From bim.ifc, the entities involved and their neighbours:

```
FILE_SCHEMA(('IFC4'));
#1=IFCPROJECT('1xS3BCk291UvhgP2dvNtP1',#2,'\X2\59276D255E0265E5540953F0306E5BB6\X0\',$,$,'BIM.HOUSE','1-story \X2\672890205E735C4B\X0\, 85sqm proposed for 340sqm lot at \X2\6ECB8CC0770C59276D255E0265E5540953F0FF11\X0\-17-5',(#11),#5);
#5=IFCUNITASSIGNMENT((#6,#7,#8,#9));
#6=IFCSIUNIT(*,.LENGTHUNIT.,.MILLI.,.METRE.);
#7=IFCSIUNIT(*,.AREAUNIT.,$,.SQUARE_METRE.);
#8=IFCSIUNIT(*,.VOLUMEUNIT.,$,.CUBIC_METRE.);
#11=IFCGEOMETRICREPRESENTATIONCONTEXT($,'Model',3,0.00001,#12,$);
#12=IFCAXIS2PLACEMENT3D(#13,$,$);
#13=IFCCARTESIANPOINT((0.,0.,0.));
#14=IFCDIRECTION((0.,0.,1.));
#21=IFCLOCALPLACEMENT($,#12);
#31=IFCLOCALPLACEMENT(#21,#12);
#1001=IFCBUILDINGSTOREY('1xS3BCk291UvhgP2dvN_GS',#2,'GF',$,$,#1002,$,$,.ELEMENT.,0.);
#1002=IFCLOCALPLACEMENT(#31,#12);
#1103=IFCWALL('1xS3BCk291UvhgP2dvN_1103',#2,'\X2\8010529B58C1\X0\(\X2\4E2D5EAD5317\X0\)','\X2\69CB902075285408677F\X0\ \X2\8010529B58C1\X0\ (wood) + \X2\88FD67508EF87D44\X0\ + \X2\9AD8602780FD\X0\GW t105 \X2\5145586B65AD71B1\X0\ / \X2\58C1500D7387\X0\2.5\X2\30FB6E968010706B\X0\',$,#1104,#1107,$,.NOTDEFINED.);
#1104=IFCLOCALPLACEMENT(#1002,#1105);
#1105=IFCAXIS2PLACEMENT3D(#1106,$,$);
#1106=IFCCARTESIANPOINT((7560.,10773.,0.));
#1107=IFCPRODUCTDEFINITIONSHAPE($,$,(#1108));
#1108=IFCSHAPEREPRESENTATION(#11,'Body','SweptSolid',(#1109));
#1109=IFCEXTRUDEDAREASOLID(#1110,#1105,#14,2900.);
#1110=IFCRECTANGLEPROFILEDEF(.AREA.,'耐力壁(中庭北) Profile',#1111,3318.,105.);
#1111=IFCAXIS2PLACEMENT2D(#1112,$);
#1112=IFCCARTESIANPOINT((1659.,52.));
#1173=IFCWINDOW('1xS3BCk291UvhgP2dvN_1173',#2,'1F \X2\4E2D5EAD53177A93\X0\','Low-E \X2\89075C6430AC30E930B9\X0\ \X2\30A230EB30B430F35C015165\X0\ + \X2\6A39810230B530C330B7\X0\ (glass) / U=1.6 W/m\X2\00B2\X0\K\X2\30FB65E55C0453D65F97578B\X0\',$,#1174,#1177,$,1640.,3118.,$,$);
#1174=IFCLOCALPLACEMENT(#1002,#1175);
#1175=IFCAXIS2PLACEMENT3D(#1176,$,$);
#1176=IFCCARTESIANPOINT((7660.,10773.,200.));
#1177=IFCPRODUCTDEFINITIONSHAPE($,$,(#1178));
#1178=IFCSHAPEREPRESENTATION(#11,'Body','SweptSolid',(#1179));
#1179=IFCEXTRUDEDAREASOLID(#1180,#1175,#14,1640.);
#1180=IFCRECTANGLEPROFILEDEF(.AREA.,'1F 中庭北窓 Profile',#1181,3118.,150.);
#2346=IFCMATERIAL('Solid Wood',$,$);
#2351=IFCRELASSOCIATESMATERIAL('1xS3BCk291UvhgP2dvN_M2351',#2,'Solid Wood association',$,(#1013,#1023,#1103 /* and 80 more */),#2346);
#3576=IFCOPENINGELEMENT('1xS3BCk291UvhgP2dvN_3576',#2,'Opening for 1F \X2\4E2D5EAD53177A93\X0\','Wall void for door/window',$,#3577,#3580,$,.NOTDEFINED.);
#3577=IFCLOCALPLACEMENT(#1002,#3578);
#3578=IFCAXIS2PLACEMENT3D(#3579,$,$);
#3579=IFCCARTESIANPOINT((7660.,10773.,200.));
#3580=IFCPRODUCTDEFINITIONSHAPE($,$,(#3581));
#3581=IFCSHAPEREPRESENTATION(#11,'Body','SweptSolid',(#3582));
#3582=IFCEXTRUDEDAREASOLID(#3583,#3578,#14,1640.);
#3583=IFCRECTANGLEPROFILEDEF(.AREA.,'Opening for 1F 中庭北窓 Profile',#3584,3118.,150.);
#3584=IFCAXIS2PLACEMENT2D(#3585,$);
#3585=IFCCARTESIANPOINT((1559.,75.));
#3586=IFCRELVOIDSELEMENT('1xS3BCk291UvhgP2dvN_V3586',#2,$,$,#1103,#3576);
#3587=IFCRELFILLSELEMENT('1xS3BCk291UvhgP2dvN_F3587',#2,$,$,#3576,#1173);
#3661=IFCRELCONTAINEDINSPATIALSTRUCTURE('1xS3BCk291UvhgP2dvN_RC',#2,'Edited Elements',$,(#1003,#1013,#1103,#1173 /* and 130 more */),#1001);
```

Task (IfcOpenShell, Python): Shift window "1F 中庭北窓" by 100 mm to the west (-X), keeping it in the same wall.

```python
import ifcopenshell
import ifcopenshell.api.geometry
import ifcopenshell.util.placement
import ifcopenshell.util.unit

model = ifcopenshell.open("bim.ifc")
unit_scale = ifcopenshell.util.unit.calculate_unit_scale(model)

window = model.by_guid("1xS3BCk291UvhgP2dvN_1173")
opening = window.FillsVoids[0].RelatingOpeningElement
wall = opening.VoidsElements[0].RelatingBuildingElement

wall_matrix = ifcopenshell.util.placement.get_local_placement(wall.ObjectPlacement)
shift = wall_matrix[:3, 0] * -0.1 / unit_scale
before = ifcopenshell.util.placement.get_local_placement(window.ObjectPlacement)[:3, 3].copy()

# The window is not placed relative to its opening, so move both.
for product in (opening, window):
    matrix = ifcopenshell.util.placement.get_local_placement(product.ObjectPlacement)
    matrix[:3, 3] += shift
    ifcopenshell.api.geometry.edit_object_placement(model, product=product, matrix=matrix, is_si=False)

after = ifcopenshell.util.placement.get_local_placement(window.ObjectPlacement)[:3, 3]
print("window moved by", (after - before).round(3) + 0.0)

model.write("bim_v2.ifc")
```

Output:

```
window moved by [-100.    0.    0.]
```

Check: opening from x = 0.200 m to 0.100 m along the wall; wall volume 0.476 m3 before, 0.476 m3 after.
